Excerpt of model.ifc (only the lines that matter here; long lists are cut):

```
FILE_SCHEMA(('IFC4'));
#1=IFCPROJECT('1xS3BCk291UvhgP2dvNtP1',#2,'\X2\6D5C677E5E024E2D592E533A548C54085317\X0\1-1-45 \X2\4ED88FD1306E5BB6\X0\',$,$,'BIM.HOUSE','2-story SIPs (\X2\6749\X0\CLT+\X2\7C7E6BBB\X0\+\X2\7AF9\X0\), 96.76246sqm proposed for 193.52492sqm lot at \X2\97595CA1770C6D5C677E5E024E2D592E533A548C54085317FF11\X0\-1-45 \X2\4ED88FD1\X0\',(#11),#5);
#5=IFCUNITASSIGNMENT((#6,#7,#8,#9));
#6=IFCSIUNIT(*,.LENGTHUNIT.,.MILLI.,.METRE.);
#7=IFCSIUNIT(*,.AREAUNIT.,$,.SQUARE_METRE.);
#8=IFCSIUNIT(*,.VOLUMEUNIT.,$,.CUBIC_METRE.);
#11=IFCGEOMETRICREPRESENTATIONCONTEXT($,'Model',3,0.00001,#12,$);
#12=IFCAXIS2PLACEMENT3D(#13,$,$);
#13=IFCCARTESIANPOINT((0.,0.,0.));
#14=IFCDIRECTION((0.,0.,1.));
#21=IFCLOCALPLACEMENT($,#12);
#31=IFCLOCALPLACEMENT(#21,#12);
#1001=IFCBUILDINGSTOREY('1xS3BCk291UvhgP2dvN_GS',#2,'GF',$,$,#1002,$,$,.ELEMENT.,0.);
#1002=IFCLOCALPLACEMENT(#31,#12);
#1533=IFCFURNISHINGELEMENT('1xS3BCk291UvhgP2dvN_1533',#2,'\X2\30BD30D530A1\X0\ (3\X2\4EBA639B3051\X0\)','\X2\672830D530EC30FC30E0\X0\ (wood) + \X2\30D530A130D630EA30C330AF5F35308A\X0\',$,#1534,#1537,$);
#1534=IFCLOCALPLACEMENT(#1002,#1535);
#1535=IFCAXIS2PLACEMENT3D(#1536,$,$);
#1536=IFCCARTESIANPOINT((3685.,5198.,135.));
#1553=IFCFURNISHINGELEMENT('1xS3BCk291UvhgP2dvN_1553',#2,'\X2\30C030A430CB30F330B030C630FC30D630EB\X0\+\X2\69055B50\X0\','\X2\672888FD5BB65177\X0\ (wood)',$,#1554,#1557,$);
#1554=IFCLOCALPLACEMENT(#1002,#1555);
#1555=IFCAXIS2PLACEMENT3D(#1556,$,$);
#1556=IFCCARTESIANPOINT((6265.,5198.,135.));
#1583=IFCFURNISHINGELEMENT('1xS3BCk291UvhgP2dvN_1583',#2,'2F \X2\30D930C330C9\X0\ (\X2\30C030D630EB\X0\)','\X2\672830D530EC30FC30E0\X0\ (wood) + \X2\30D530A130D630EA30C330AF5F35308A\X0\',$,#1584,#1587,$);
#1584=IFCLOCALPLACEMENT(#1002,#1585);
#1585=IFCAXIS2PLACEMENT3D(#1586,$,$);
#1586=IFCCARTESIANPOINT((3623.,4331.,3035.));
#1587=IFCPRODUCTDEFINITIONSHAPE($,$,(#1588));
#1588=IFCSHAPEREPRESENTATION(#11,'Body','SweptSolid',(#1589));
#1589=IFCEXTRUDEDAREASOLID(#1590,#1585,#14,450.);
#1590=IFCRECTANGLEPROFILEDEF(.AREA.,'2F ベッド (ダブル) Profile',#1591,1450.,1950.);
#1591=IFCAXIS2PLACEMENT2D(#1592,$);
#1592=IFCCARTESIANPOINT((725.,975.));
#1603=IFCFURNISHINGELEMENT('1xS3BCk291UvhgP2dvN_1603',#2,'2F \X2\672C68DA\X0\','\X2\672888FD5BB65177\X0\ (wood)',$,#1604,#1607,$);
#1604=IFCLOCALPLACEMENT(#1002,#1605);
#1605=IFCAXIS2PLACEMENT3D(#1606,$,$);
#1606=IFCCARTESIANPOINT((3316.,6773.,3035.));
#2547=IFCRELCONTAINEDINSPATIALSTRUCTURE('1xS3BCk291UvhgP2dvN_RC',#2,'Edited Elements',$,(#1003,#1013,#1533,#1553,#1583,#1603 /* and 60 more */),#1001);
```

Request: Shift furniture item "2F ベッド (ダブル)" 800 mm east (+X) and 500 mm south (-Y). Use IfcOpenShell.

```python
import ifcopenshell
import ifcopenshell.api.geometry
import ifcopenshell.util.placement

model = ifcopenshell.open("model.ifc")

item = model.by_guid("1xS3BCk291UvhgP2dvN_1583")
matrix = ifcopenshell.util.placement.get_local_placement(item.ObjectPlacement)
matrix[0, 3] += 800.0
matrix[1, 3] -= 500.0
ifcopenshell.api.geometry.edit_object_placement(model, product=item, matrix=matrix, is_si=False)

print(ifcopenshell.util.placement.get_local_placement(item.ObjectPlacement).round(3) + 0.0)

model.write("model_edited.ifc")
```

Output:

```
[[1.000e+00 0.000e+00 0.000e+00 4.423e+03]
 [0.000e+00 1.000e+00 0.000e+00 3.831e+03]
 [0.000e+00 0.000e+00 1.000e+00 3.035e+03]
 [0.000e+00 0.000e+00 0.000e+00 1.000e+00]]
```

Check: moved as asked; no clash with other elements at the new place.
